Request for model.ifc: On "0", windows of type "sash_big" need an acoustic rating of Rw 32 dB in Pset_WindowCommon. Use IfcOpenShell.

First a look at what the model holds.

```python
import ifcopenshell
import ifcopenshell.util.element

model = ifcopenshell.open("model.ifc")
print(model.schema)
storey = next(s for s in model.by_type("IfcBuildingStorey") if s.Name == "0")
windows = [e for e in ifcopenshell.util.element.get_decomposition(storey) if e.is_a("IfcWindow")]
seen = {}
for e in windows:
    element_type = ifcopenshell.util.element.get_type(e)
    key = (element_type.Name if element_type != e and element_type else None, ifcopenshell.util.element.get_pset(e, "Pset_WindowCommon", "AcousticRating"))
    seen[key] = seen.get(key, 0) + 1
for (name, value), count in sorted(seen.items(), key=str):
    print(count, "x", name, "|", value)
```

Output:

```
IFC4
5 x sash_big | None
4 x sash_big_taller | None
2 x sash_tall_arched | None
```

```python
import ifcopenshell
import ifcopenshell.api.pset
import ifcopenshell.util.element

model = ifcopenshell.open("model.ifc")

storey = next(s for s in model.by_type("IfcBuildingStorey") if s.Name == "0")
windows = [e for e in ifcopenshell.util.element.get_decomposition(storey) if e.is_a("IfcWindow")]

count = 0
for e in windows:
    element_type = ifcopenshell.util.element.get_type(e)
    if element_type in (None, e) or element_type.Name != "sash_big":
        continue
    # add_pset returns the element's existing set when there is one.
    pset = ifcopenshell.api.pset.add_pset(model, product=e, name="Pset_WindowCommon")
    ifcopenshell.api.pset.edit_pset(model, pset=pset, properties={"AcousticRating": "Rw 32 dB"})
    count += 1

print(count, "windows updated")

model.write("model-out.ifc")
```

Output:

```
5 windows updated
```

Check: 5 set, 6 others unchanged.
